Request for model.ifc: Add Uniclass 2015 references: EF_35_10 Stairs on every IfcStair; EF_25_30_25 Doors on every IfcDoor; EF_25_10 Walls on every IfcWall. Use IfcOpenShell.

First a look at what the model holds.

```python
import ifcopenshell

model = ifcopenshell.open("model.ifc")
print(model.schema)
print("classifications:", [c.Name for c in model.by_type("IfcClassification")])
for ifc_class in ("IfcDoor", "IfcRoof", "IfcStair", "IfcWall", "IfcWindow"):
    print(ifc_class, len(model.by_type(ifc_class)))
```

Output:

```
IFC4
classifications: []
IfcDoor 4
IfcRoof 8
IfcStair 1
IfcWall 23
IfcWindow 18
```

```python
import ifcopenshell
import ifcopenshell.api.classification

model = ifcopenshell.open("model.ifc")

system = ifcopenshell.api.classification.add_classification(model, classification="Uniclass 2015")

codes = {
    "IfcStair": ("EF_35_10", "Stairs"),
    "IfcDoor": ("EF_25_30_25", "Doors"),
    "IfcWall": ("EF_25_10", "Walls"),
}
for ifc_class, (code, name) in codes.items():
    products = model.by_type(ifc_class)
    ifcopenshell.api.classification.add_reference(
        model, products=products, classification=system, identification=code, name=name
    )
    print(code, len(products))

model.write("model_v2.ifc")
```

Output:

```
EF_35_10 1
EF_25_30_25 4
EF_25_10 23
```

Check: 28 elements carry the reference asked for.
